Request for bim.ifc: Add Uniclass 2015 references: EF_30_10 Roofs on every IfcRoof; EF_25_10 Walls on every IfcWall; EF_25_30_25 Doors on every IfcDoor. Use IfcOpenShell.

First a look at what the model holds.

```python
import ifcopenshell

model = ifcopenshell.open("bim.ifc")
print(model.schema)
print("classifications:", [c.Name for c in model.by_type("IfcClassification")])
for ifc_class in ("IfcDoor", "IfcRoof", "IfcStair", "IfcWall", "IfcWindow"):
    print(ifc_class, len(model.by_type(ifc_class)))
```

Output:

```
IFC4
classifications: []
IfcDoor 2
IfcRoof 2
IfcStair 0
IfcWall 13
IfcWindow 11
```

```python
import ifcopenshell
import ifcopenshell.api.classification

model = ifcopenshell.open("bim.ifc")

system = ifcopenshell.api.classification.add_classification(model, classification="Uniclass 2015")

codes = {
    "IfcRoof": ("EF_30_10", "Roofs"),
    "IfcWall": ("EF_25_10", "Walls"),
    "IfcDoor": ("EF_25_30_25", "Doors"),
}
for ifc_class, (code, name) in codes.items():
    products = model.by_type(ifc_class)
    ifcopenshell.api.classification.add_reference(
        model, products=products, classification=system, identification=code, name=name
    )
    print(code, len(products))

model.write("bim-out.ifc")
```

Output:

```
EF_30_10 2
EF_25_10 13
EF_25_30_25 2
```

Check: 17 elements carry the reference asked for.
